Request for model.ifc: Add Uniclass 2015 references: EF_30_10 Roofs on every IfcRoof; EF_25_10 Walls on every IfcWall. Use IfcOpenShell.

First a look at what the model holds.

```python
import ifcopenshell

model = ifcopenshell.open("model.ifc")
print(model.schema)
print("classifications:", [c.Name for c in model.by_type("IfcClassification")])
for ifc_class in ("IfcDoor", "IfcRoof", "IfcStair", "IfcWall", "IfcWindow"):
    print(ifc_class, len(model.by_type(ifc_class)))
```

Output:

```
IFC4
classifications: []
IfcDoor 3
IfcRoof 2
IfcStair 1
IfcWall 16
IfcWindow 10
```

```python
import ifcopenshell
import ifcopenshell.api.classification

model = ifcopenshell.open("model.ifc")

system = ifcopenshell.api.classification.add_classification(model, classification="Uniclass 2015")

codes = {
    "IfcRoof": ("EF_30_10", "Roofs"),
    "IfcWall": ("EF_25_10", "Walls"),
}
for ifc_class, (code, name) in codes.items():
    products = model.by_type(ifc_class)
    ifcopenshell.api.classification.add_reference(
        model, products=products, classification=system, identification=code, name=name
    )
    print(code, len(products))

model.write("model_updated.ifc")
```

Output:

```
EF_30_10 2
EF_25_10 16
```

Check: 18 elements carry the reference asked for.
